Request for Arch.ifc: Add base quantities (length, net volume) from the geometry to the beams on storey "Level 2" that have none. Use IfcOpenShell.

First a look at what the model holds.

```python
import ifcopenshell
import ifcopenshell.util.element
import ifcopenshell.util.unit

model = ifcopenshell.open("Arch.ifc")
print(model.schema)
for unit_type in ("LENGTHUNIT", "AREAUNIT", "VOLUMEUNIT"):
    print(unit_type, ifcopenshell.util.unit.calculate_unit_scale(model, unit_type))
storey = next(s for s in model.by_type("IfcBuildingStorey") if s.Name == "Level 2")
beams = [e for e in ifcopenshell.util.element.get_decomposition(storey) if e.is_a("IfcBeam")]
for e in sorted(beams, key=lambda e: e.id()):
    print(e.id(), e.is_a(), e.Name, list(ifcopenshell.util.element.get_psets(e, qtos_only=True)), sep=" | ")
```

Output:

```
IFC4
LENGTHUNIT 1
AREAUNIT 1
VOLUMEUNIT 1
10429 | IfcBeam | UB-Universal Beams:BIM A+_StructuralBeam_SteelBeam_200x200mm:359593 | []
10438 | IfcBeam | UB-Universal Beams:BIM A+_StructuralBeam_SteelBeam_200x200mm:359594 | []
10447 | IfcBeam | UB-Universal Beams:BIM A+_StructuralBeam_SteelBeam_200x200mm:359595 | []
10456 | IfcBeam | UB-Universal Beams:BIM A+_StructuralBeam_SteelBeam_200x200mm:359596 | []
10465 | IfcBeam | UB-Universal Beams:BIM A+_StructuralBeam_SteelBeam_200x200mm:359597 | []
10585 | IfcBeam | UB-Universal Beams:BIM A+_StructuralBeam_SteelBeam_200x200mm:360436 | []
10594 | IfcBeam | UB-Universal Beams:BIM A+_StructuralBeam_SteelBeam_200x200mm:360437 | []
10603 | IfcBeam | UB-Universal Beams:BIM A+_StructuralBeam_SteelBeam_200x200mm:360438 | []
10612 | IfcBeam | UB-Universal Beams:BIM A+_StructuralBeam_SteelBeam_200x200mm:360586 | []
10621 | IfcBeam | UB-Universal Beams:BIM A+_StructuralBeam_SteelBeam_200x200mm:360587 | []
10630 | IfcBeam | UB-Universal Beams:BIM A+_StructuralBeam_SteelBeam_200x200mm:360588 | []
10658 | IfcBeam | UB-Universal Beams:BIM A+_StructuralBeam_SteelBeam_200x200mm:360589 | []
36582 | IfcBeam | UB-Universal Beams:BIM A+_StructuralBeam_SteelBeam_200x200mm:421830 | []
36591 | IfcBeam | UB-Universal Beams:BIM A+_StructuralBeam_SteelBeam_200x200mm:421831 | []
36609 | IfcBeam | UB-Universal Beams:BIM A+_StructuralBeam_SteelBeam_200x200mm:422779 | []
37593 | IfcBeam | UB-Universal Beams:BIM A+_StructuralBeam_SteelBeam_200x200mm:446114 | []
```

```python
import ifcopenshell
import ifcopenshell.api.pset
import ifcopenshell.geom
import ifcopenshell.util.element
import ifcopenshell.util.shape
import ifcopenshell.util.unit

model = ifcopenshell.open("Arch.ifc")
unit_scale = ifcopenshell.util.unit.calculate_unit_scale(model)
volume_scale = ifcopenshell.util.unit.calculate_unit_scale(model, "VOLUMEUNIT")
settings = ifcopenshell.geom.settings()

storey = next(s for s in model.by_type("IfcBuildingStorey") if s.Name == "Level 2")
beams = [e for e in ifcopenshell.util.element.get_decomposition(storey) if e.is_a("IfcBeam")]

for e in sorted(beams, key=lambda e: e.id()):
    if ifcopenshell.util.element.get_psets(e, qtos_only=True, should_inherit=False):
        continue
    # Geometry comes back in metres, in the element's own axes.
    shape = ifcopenshell.geom.create_shape(settings, e)
    values = {
        "Length": ifcopenshell.util.shape.get_max_xyz(shape.geometry) / unit_scale,
        "NetVolume": ifcopenshell.util.shape.get_volume(shape.geometry) / volume_scale,
    }
    qto = ifcopenshell.api.pset.add_qto(model, product=e, name="Qto_BeamBaseQuantities")
    ifcopenshell.api.pset.edit_qto(model, qto=qto, properties=values)
    print(e.id(), {k: round(v, 3) for k, v in values.items()})

model.write("Arch_edited.ifc")
```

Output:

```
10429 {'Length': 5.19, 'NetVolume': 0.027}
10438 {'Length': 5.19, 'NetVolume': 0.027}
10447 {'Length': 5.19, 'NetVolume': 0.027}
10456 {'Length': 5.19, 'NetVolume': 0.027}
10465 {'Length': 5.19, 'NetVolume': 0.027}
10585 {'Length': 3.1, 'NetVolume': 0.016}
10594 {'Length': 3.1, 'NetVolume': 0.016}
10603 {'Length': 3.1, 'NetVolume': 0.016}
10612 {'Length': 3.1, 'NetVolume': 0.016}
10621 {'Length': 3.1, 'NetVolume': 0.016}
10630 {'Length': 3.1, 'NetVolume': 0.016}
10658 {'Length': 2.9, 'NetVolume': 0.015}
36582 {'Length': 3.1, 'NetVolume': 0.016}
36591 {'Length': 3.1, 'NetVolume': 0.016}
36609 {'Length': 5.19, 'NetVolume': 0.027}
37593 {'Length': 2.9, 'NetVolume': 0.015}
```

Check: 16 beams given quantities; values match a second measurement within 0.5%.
